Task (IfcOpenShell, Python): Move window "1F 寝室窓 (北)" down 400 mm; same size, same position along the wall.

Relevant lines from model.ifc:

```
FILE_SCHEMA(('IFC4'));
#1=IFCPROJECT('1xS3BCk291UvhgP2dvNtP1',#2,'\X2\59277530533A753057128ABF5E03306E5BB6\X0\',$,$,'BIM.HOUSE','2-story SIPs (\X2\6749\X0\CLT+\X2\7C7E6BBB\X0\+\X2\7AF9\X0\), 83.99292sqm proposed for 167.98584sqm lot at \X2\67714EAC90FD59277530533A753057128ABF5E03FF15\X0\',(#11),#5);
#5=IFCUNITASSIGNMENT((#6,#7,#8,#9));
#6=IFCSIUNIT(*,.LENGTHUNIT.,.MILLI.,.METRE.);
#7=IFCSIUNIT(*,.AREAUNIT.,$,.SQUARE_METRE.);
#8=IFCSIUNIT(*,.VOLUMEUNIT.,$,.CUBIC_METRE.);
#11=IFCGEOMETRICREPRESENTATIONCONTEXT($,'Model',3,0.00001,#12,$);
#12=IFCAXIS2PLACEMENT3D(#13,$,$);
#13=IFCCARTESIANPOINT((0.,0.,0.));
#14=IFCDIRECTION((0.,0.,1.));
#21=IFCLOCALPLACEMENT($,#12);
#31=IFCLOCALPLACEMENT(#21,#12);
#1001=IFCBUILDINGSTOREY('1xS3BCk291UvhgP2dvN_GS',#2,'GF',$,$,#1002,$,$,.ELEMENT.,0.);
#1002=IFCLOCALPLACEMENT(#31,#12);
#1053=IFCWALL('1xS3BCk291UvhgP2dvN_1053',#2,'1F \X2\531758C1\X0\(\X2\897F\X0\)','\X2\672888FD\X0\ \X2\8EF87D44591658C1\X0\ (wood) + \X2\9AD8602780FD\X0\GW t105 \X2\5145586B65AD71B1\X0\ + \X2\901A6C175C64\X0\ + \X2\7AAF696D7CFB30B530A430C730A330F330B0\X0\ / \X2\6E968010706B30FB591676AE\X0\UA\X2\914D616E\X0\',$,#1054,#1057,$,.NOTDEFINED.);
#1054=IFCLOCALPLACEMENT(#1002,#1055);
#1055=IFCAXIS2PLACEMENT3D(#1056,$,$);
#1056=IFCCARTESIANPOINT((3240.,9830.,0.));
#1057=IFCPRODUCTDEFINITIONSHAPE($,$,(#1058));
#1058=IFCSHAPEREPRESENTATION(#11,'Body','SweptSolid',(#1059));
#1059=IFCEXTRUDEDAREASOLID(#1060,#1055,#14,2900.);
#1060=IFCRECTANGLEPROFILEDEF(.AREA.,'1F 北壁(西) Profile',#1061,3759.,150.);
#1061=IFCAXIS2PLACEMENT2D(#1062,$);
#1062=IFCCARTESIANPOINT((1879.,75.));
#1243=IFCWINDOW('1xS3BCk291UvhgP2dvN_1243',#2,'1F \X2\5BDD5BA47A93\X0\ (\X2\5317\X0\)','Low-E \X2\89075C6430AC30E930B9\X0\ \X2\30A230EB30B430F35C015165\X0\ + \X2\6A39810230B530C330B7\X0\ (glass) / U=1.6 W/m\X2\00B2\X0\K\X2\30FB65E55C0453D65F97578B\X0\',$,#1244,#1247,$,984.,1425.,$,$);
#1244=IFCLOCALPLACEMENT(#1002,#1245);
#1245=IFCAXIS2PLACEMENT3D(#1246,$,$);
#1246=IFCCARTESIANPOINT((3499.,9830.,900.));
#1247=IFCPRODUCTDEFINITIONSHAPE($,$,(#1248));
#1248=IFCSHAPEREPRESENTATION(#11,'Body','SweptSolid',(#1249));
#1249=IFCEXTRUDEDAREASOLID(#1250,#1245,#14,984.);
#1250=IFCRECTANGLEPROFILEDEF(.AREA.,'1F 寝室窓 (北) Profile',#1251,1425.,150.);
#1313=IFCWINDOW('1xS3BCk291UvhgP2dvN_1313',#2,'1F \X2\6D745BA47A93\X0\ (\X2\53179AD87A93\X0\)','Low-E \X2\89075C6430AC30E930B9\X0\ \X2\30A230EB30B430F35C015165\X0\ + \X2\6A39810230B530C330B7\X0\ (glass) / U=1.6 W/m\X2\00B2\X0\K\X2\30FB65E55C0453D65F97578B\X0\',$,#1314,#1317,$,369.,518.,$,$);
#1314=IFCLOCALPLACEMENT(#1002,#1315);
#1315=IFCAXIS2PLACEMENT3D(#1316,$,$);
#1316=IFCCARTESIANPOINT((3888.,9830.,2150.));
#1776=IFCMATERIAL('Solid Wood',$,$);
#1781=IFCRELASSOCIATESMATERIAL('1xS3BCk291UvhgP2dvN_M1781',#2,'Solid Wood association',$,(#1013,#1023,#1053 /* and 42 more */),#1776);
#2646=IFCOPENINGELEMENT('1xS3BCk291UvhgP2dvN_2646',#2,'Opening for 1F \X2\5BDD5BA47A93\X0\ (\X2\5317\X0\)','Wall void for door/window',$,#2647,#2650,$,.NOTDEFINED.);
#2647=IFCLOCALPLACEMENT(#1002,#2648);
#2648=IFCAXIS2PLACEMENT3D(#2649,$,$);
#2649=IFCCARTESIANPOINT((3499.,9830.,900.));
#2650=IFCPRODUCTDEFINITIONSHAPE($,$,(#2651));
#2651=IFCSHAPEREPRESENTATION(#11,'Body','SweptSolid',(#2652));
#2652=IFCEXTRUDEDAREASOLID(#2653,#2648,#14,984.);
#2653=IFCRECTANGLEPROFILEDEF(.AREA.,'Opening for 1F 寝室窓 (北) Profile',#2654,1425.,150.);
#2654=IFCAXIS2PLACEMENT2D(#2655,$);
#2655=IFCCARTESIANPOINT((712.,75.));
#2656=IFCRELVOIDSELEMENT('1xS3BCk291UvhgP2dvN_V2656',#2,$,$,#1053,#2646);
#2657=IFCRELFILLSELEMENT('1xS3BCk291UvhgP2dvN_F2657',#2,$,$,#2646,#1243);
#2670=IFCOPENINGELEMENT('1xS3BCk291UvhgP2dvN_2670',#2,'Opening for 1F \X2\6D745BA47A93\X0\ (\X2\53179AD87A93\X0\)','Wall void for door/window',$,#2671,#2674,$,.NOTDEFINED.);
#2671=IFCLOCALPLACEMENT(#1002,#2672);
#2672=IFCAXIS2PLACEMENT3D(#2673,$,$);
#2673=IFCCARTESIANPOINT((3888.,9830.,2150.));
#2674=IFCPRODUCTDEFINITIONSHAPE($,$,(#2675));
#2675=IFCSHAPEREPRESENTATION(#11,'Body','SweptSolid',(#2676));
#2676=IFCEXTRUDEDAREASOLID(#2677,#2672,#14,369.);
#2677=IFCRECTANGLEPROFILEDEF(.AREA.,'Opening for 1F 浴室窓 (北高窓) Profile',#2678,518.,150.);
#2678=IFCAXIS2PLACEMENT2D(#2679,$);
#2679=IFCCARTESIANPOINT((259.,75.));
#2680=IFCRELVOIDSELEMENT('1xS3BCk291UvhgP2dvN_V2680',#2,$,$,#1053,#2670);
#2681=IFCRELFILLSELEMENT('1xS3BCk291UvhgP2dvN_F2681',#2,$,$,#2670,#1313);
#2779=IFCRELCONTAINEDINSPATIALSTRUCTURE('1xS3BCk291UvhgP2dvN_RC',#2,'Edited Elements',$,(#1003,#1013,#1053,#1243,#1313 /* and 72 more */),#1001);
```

```python
import numpy as np
import ifcopenshell
import ifcopenshell.api.geometry
import ifcopenshell.util.placement
import ifcopenshell.util.unit

model = ifcopenshell.open("model.ifc")
unit_scale = ifcopenshell.util.unit.calculate_unit_scale(model)

window = model.by_guid("1xS3BCk291UvhgP2dvN_1243")
opening = window.FillsVoids[0].RelatingOpeningElement
dz = -0.4 / unit_scale

shift = np.array([0.0, 0.0, dz])
# The window is not placed relative to its opening, so move both.
for product in (opening, window):
    matrix = ifcopenshell.util.placement.get_local_placement(product.ObjectPlacement)
    matrix[:3, 3] += shift
    ifcopenshell.api.geometry.edit_object_placement(model, product=product, matrix=matrix, is_si=False)

print(f"moved by {dz * unit_scale:+.3f} m")

model.write("model_rev.ifc")
```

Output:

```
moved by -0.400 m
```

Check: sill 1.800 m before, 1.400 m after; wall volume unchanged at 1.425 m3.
